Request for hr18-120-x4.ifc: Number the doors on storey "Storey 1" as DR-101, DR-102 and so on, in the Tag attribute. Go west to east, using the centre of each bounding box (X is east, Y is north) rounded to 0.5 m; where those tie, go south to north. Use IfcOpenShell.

First a look at what the model holds.

```python
import ifcopenshell
import ifcopenshell.util.element
import ifcopenshell.util.placement

model = ifcopenshell.open("hr18-120-x4.ifc")
print(model.schema)
storey = next(s for s in model.by_type("IfcBuildingStorey") if s.Name == "Storey 1")
doors = [e for e in ifcopenshell.util.element.get_decomposition(storey) if e.is_a("IfcDoor")]
for e in sorted(doors, key=lambda e: e.id()):
    origin = ifcopenshell.util.placement.get_local_placement(e.ObjectPlacement)[:3, 3]
    print(e.id(), e.Tag, e.Name, origin.round(2) + 0.0, sep=" | ")
```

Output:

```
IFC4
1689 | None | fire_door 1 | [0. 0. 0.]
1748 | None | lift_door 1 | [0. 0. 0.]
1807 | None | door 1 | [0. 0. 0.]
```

```python
import ifcopenshell
import ifcopenshell.geom
import ifcopenshell.util.element
import ifcopenshell.util.shape

model = ifcopenshell.open("hr18-120-x4.ifc")
settings = ifcopenshell.geom.settings()
settings.set("use-world-coords", True)


def centre(element):
    shape = ifcopenshell.geom.create_shape(settings, element)
    return ifcopenshell.util.shape.get_bbox_centroid(shape.geometry)


storey = next(s for s in model.by_type("IfcBuildingStorey") if s.Name == "Storey 1")
doors = [e for e in ifcopenshell.util.element.get_decomposition(storey) if e.is_a("IfcDoor")]

# Insertion points can sit at a corner or the storey origin, so sort by the geometry (in metres).
centres = {e: centre(e) for e in doors}
doors.sort(key=lambda e: (round(centres[e][0] / 0.5), centres[e][1]))

for i, e in enumerate(doors, start=1):
    number = f"DR-1{i:02d}"
    e.Tag = number
    print(e.id(), number)

model.write("hr18-120-x4_v2.ifc")
```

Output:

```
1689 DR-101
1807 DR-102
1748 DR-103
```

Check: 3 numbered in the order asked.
